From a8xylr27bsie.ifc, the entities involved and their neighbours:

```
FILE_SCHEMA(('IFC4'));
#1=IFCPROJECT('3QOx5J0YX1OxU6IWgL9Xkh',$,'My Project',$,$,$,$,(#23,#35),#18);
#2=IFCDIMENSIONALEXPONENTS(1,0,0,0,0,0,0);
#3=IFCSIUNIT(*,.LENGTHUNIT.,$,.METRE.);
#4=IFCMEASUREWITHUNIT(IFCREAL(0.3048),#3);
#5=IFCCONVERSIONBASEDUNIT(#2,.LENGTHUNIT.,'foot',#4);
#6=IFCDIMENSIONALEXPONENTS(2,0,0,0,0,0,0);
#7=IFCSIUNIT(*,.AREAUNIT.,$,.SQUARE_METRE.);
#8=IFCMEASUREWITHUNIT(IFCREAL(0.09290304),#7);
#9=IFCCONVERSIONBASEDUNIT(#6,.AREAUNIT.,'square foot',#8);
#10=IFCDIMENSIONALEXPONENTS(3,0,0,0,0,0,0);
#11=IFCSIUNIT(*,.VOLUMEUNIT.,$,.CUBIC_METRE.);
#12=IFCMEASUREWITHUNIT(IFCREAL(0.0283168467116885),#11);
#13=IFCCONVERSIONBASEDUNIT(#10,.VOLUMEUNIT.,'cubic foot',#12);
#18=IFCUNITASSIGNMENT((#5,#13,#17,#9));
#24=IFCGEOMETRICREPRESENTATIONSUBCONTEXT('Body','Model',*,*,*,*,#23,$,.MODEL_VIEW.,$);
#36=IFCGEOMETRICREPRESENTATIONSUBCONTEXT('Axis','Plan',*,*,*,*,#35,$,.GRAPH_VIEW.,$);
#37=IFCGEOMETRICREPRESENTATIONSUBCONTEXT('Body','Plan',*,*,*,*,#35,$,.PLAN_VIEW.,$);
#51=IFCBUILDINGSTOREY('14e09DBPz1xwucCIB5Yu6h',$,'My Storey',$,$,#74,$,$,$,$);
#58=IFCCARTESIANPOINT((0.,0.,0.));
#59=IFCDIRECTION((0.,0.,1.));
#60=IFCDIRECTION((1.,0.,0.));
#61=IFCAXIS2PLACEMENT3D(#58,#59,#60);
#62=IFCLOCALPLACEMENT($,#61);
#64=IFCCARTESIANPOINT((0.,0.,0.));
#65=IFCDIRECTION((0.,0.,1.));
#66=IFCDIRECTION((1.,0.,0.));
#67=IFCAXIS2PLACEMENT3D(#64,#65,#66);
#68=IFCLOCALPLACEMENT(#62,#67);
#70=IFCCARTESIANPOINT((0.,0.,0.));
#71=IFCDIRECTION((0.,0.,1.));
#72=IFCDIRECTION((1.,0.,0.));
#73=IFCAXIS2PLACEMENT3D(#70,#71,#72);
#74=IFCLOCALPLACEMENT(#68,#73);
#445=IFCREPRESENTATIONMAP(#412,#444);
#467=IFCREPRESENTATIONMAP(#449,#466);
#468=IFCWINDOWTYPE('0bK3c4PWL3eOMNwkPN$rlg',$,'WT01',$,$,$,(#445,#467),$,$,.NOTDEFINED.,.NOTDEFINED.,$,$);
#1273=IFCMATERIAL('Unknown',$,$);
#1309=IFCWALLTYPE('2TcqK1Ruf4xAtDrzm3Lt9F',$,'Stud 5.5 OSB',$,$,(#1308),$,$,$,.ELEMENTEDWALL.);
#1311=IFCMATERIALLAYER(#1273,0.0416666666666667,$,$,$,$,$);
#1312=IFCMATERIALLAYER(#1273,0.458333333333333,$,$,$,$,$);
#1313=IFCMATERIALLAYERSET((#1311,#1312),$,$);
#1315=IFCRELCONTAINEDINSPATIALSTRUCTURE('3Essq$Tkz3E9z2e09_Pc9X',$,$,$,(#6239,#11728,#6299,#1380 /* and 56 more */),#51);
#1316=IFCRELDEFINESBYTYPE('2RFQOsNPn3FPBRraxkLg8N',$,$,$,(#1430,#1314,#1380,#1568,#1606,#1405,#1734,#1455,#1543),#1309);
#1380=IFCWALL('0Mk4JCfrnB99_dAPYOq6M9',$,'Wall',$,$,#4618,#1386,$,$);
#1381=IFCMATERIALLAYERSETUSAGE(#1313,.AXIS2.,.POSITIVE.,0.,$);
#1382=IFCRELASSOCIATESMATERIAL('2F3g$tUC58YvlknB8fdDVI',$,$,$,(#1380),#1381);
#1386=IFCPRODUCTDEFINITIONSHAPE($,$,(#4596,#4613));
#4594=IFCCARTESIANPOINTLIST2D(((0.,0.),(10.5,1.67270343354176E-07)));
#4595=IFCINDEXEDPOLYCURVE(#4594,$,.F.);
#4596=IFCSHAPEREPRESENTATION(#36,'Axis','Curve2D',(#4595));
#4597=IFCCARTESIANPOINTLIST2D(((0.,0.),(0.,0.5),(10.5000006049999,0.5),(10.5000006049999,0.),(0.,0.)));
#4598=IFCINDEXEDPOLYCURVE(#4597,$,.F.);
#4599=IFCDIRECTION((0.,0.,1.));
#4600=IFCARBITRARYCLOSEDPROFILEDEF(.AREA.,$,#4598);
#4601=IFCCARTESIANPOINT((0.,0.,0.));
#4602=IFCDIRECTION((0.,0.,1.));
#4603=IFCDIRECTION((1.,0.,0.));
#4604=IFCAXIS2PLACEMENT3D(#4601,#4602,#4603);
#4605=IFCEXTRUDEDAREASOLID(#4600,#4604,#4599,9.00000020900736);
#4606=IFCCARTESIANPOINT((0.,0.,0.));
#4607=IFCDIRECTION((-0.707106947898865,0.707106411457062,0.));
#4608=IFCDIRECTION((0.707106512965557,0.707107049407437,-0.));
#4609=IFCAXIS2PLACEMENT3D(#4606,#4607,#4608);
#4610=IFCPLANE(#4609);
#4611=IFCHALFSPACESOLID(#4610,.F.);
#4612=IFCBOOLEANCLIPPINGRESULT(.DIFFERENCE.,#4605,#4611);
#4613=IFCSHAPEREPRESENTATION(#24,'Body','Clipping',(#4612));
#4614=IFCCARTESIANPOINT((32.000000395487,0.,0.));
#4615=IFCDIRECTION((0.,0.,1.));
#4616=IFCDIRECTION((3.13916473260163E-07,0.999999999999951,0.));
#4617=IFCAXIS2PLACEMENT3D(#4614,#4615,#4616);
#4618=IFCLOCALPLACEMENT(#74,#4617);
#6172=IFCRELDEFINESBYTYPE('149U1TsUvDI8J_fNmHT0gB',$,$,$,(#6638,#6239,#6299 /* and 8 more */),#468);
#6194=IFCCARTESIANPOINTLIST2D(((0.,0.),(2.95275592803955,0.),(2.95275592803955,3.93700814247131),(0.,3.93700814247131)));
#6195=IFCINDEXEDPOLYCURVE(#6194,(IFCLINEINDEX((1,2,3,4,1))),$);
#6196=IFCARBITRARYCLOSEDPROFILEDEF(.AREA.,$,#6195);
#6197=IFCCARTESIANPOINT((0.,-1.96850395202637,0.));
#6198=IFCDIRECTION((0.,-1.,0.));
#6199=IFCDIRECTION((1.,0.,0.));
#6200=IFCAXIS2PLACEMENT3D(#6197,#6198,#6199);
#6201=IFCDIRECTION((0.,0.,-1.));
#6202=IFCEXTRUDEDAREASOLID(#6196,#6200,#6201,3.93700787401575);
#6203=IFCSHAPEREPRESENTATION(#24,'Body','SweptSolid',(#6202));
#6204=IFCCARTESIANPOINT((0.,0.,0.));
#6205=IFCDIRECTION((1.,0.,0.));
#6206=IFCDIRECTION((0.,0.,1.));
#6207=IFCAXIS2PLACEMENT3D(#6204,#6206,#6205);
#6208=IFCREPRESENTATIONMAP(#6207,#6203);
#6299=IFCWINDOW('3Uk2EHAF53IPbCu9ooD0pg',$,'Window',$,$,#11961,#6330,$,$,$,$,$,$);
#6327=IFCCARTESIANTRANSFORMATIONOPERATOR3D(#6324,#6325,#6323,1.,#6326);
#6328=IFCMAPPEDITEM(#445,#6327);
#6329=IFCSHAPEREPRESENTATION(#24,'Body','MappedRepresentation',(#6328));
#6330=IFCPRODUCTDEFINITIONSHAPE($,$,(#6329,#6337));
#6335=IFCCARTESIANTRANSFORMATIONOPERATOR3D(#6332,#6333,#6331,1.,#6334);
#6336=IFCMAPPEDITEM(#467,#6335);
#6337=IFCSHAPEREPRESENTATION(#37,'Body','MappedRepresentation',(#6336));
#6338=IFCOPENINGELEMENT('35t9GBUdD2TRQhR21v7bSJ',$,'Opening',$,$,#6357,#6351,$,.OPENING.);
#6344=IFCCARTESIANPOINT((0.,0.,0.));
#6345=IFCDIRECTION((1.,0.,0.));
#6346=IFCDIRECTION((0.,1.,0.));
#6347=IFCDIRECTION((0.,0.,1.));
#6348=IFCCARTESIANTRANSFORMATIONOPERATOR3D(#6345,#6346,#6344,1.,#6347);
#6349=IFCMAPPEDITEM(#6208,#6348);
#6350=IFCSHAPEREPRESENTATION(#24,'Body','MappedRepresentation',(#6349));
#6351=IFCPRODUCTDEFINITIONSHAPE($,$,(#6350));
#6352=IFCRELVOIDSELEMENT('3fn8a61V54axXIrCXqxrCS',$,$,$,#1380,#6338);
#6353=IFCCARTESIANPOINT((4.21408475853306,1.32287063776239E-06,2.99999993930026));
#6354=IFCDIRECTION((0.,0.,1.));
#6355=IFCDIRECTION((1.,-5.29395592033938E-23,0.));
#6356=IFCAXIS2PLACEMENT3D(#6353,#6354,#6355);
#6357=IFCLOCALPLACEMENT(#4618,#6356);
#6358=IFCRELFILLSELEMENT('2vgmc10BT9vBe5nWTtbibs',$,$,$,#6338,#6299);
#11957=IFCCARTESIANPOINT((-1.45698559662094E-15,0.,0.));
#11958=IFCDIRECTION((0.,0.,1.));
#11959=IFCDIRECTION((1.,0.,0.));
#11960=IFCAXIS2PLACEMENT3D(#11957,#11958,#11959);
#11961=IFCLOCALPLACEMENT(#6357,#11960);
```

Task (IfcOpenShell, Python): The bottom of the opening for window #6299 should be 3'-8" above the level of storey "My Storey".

```python
import numpy as np
import ifcopenshell
import ifcopenshell.api.geometry
import ifcopenshell.geom
import ifcopenshell.util.element
import ifcopenshell.util.placement
import ifcopenshell.util.shape
import ifcopenshell.util.unit

model = ifcopenshell.open("a8xylr27bsie.ifc")
unit_scale = ifcopenshell.util.unit.calculate_unit_scale(model)

window = model.by_id(6299)
opening = window.FillsVoids[0].RelatingOpeningElement
storey = ifcopenshell.util.element.get_container(window, ifc_class="IfcBuildingStorey")
level = ifcopenshell.util.placement.get_local_placement(storey.ObjectPlacement)[2, 3]

# The opening's origin need not be at the sill, so measure its lowest point.
shape = ifcopenshell.geom.create_shape(ifcopenshell.geom.settings(), opening)
bottom = ifcopenshell.util.shape.get_shape_bottom_elevation(shape, shape.geometry) / unit_scale
dz = level + 44 * 0.0254 / unit_scale - bottom

shift = np.array([0.0, 0.0, dz])
# The window is placed relative to its opening, so it follows when the opening moves.
matrix = ifcopenshell.util.placement.get_local_placement(opening.ObjectPlacement)
matrix[:3, 3] += shift
ifcopenshell.api.geometry.edit_object_placement(
    model, product=opening, matrix=matrix, is_si=False, should_transform_children=True
)

print(f"moved by {dz * unit_scale:+.3f} m")

model.write("a8xylr27bsie_rev.ifc")
```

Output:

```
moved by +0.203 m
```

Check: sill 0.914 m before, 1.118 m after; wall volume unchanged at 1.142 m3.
